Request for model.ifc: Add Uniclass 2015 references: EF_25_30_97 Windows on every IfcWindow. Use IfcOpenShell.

First a look at what the model holds.

```python
import ifcopenshell

model = ifcopenshell.open("model.ifc")
print(model.schema)
print("classifications:", [c.Name for c in model.by_type("IfcClassification")])
for ifc_class in ("IfcDoor", "IfcRoof", "IfcStair", "IfcWall", "IfcWindow"):
    print(ifc_class, len(model.by_type(ifc_class)))
```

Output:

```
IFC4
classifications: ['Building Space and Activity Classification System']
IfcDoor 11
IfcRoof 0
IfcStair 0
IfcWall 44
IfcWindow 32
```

```python
import ifcopenshell
import ifcopenshell.api.classification

model = ifcopenshell.open("model.ifc")

system = ifcopenshell.api.classification.add_classification(model, classification="Uniclass 2015")

codes = {
    "IfcWindow": ("EF_25_30_97", "Windows"),
}
for ifc_class, (code, name) in codes.items():
    products = model.by_type(ifc_class)
    ifcopenshell.api.classification.add_reference(
        model, products=products, classification=system, identification=code, name=name
    )
    print(code, len(products))

model.write("model-out.ifc")
```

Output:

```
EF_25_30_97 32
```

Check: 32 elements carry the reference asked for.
